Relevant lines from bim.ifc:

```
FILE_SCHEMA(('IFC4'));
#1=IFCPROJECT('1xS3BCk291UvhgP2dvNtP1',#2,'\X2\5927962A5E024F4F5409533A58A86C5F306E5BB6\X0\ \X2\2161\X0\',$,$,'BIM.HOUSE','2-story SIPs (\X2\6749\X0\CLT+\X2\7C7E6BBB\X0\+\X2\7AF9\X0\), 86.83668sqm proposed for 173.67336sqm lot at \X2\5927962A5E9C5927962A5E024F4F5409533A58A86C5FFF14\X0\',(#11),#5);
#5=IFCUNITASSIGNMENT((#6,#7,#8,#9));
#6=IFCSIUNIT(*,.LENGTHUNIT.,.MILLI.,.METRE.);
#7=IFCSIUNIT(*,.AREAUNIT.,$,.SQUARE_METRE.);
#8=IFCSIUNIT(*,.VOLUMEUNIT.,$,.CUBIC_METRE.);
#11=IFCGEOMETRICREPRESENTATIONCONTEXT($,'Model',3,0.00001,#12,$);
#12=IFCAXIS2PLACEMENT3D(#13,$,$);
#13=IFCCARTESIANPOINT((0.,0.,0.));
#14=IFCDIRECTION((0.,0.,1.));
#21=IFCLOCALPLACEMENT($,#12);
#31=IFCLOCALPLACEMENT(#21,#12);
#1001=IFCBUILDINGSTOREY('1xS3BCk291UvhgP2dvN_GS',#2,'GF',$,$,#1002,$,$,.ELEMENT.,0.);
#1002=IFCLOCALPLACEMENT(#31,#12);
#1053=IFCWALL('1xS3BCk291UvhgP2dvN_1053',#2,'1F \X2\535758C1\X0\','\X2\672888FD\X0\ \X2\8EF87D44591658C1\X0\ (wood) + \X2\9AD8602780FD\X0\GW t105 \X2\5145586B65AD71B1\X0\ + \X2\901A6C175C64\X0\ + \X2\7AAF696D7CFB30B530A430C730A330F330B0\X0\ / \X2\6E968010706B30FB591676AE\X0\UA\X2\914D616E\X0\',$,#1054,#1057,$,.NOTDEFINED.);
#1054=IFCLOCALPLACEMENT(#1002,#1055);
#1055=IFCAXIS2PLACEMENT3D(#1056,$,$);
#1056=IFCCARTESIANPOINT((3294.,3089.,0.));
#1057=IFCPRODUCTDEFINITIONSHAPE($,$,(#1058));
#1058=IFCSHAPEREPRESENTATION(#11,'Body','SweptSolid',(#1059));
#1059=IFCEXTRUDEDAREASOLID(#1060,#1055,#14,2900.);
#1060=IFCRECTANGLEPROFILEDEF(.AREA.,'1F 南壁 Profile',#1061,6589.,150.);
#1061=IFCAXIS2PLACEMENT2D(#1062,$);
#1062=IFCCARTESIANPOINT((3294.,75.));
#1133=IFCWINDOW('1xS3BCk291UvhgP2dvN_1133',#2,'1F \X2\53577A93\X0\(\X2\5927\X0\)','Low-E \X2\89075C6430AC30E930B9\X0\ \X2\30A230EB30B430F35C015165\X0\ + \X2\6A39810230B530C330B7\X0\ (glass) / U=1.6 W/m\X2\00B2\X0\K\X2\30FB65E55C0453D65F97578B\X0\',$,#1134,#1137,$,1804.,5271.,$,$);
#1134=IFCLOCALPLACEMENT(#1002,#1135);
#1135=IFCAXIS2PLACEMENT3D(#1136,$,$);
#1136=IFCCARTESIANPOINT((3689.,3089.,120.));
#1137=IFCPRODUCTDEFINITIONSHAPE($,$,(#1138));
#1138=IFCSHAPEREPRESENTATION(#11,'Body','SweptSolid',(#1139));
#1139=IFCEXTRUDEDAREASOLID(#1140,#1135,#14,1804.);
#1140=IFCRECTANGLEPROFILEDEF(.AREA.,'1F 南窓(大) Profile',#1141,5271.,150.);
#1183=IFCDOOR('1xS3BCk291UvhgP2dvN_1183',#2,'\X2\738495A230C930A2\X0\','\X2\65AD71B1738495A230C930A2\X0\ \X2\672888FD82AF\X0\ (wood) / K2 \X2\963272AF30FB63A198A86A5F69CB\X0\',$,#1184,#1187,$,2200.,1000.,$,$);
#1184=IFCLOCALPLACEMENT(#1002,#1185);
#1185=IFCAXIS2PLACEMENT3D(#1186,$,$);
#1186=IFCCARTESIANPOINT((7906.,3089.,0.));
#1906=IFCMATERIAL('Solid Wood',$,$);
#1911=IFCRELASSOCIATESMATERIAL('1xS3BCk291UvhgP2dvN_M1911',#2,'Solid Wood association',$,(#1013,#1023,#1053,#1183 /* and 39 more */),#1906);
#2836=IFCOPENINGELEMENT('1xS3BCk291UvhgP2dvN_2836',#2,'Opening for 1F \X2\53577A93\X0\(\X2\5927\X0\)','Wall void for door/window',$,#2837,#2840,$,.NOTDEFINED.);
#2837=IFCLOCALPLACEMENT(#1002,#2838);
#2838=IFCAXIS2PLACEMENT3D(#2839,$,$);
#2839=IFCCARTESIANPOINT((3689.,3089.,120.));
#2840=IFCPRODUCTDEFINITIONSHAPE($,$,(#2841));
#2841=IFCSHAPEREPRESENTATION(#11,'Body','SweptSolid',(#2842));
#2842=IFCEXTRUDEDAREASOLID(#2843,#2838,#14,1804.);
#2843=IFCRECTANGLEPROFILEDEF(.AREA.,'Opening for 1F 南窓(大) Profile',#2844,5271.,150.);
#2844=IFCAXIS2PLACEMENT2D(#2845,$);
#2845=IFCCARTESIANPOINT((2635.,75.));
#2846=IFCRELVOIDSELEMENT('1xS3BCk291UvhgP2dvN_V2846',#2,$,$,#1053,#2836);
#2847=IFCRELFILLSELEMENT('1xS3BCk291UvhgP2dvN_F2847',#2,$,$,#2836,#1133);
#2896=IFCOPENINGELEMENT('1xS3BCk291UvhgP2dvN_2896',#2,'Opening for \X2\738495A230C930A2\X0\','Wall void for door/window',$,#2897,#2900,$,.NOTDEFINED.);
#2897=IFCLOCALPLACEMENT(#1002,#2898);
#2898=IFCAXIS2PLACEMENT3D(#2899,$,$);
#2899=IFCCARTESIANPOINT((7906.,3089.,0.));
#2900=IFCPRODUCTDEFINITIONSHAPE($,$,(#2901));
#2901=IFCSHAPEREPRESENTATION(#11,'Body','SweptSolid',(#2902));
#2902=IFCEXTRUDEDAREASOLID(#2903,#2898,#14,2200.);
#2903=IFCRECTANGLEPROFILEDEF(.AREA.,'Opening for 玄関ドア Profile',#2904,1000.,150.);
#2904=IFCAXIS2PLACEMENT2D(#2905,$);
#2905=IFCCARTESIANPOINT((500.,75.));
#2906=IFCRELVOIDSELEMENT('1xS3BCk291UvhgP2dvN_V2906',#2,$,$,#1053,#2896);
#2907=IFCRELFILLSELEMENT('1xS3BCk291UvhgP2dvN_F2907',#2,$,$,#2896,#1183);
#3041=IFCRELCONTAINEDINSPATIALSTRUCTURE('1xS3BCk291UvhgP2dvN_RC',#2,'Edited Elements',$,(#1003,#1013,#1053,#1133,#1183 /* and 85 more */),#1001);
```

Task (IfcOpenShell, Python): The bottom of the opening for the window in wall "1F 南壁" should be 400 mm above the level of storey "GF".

```python
import numpy as np
import ifcopenshell
import ifcopenshell.api.geometry
import ifcopenshell.geom
import ifcopenshell.util.element
import ifcopenshell.util.placement
import ifcopenshell.util.shape
import ifcopenshell.util.unit

model = ifcopenshell.open("bim.ifc")
unit_scale = ifcopenshell.util.unit.calculate_unit_scale(model)

window = model.by_guid("1xS3BCk291UvhgP2dvN_1133")
opening = window.FillsVoids[0].RelatingOpeningElement
storey = ifcopenshell.util.element.get_container(window, ifc_class="IfcBuildingStorey")
level = ifcopenshell.util.placement.get_local_placement(storey.ObjectPlacement)[2, 3]

# The opening's origin need not be at the sill, so measure its lowest point.
shape = ifcopenshell.geom.create_shape(ifcopenshell.geom.settings(), opening)
bottom = ifcopenshell.util.shape.get_shape_bottom_elevation(shape, shape.geometry) / unit_scale
dz = level + 400.0 - bottom

shift = np.array([0.0, 0.0, dz])
# The window is not placed relative to its opening, so move both.
for product in (opening, window):
    matrix = ifcopenshell.util.placement.get_local_placement(product.ObjectPlacement)
    matrix[:3, 3] += shift
    ifcopenshell.api.geometry.edit_object_placement(model, product=product, matrix=matrix, is_si=False)

print(f"moved by {dz * unit_scale:+.3f} m")

model.write("bim_v2.ifc")
```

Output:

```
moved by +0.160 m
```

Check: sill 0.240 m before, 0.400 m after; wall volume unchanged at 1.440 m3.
